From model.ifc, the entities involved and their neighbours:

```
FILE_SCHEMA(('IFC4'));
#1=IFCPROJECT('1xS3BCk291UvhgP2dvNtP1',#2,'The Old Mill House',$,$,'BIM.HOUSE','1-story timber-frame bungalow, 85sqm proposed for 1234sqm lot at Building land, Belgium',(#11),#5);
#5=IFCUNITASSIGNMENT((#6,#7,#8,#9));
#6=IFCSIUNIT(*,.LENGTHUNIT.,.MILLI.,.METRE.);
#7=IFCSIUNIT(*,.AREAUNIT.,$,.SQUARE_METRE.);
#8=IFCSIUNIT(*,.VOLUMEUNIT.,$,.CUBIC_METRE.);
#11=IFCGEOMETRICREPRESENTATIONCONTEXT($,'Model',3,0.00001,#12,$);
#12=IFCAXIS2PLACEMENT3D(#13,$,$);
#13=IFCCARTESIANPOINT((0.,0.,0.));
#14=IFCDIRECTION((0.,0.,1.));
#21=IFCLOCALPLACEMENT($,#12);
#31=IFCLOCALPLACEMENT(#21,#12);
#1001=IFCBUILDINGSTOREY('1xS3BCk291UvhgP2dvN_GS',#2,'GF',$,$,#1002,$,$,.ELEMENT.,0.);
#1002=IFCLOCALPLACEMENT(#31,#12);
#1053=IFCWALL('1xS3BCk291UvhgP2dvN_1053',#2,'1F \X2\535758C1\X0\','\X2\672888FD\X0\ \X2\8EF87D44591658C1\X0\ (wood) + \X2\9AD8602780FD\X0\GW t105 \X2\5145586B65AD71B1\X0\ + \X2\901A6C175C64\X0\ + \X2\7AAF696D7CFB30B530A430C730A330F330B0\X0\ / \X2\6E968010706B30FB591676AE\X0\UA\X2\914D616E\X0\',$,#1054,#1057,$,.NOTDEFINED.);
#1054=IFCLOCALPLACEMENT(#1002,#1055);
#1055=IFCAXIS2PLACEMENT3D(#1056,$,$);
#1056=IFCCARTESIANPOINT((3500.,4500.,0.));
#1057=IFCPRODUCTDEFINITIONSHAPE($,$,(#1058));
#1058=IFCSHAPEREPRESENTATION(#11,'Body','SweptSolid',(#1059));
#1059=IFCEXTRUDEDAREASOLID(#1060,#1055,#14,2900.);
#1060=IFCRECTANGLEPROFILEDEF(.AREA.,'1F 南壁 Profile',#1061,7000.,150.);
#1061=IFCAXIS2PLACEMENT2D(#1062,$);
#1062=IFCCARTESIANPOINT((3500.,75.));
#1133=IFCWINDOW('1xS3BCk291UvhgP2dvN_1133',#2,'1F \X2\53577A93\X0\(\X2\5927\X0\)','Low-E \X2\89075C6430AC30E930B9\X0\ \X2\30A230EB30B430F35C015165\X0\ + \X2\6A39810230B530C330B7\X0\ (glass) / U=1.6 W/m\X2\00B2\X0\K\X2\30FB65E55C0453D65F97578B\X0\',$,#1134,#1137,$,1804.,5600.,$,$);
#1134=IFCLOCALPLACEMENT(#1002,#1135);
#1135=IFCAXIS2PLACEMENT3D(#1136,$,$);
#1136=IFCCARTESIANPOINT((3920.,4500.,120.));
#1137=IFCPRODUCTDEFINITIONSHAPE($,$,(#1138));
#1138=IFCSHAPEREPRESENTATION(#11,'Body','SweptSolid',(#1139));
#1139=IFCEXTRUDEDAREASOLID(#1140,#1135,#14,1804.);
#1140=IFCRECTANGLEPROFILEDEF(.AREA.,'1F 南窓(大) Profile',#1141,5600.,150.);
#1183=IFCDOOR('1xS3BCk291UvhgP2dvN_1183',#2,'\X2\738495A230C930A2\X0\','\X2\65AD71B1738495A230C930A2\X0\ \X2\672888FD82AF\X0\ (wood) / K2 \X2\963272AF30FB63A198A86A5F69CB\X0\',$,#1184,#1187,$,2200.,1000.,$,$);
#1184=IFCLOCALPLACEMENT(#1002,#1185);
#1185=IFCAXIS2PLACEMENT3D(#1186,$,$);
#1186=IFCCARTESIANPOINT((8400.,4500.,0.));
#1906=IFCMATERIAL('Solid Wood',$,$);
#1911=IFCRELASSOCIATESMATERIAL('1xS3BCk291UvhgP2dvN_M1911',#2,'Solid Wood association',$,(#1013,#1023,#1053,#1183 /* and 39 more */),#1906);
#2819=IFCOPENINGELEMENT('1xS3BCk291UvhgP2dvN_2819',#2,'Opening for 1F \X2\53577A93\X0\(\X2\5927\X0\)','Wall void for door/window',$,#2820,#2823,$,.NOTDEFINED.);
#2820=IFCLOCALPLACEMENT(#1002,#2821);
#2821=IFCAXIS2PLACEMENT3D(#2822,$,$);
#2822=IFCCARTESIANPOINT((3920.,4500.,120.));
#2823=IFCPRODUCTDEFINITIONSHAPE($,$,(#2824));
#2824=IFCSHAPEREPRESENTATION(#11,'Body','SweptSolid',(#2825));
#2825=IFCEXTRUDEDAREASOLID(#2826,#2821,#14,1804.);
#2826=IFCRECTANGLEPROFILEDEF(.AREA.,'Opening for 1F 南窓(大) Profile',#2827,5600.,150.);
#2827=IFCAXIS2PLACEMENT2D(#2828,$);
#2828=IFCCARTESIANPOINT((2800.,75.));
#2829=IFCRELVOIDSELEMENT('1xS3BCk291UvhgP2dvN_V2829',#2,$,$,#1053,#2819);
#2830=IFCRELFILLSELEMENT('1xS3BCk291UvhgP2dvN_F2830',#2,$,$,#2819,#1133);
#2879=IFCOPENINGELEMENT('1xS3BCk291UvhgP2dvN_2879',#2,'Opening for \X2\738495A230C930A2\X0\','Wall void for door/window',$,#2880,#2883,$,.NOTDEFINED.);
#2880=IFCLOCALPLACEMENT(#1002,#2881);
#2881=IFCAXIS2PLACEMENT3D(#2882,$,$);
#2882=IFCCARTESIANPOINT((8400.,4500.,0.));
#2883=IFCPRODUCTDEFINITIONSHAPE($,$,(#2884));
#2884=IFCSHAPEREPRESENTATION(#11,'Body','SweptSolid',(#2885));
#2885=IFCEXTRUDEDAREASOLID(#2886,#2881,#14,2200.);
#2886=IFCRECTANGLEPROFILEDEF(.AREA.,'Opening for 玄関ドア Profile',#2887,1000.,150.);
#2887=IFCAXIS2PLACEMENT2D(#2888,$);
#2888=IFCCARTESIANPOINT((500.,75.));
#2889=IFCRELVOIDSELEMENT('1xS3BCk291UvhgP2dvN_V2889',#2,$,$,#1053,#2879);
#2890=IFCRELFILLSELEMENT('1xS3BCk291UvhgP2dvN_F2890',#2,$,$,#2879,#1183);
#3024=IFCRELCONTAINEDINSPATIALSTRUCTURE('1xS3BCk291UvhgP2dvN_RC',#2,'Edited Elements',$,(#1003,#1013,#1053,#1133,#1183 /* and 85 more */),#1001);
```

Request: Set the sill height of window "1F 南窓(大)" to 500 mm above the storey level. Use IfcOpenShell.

```python
import numpy as np
import ifcopenshell
import ifcopenshell.api.geometry
import ifcopenshell.geom
import ifcopenshell.util.element
import ifcopenshell.util.placement
import ifcopenshell.util.shape
import ifcopenshell.util.unit

model = ifcopenshell.open("model.ifc")
unit_scale = ifcopenshell.util.unit.calculate_unit_scale(model)

window = model.by_guid("1xS3BCk291UvhgP2dvN_1133")
opening = window.FillsVoids[0].RelatingOpeningElement
storey = ifcopenshell.util.element.get_container(window, ifc_class="IfcBuildingStorey")
level = ifcopenshell.util.placement.get_local_placement(storey.ObjectPlacement)[2, 3]

# The opening's origin need not be at the sill, so measure its lowest point.
shape = ifcopenshell.geom.create_shape(ifcopenshell.geom.settings(), opening)
bottom = ifcopenshell.util.shape.get_shape_bottom_elevation(shape, shape.geometry) / unit_scale
dz = level + 500.0 - bottom

shift = np.array([0.0, 0.0, dz])
# The window is not placed relative to its opening, so move both.
for product in (opening, window):
    matrix = ifcopenshell.util.placement.get_local_placement(product.ObjectPlacement)
    matrix[:3, 3] += shift
    ifcopenshell.api.geometry.edit_object_placement(model, product=product, matrix=matrix, is_si=False)

print(f"moved by {dz * unit_scale:+.3f} m")

model.write("model_rev.ifc")
```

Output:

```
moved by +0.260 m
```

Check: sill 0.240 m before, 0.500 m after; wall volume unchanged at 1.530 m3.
